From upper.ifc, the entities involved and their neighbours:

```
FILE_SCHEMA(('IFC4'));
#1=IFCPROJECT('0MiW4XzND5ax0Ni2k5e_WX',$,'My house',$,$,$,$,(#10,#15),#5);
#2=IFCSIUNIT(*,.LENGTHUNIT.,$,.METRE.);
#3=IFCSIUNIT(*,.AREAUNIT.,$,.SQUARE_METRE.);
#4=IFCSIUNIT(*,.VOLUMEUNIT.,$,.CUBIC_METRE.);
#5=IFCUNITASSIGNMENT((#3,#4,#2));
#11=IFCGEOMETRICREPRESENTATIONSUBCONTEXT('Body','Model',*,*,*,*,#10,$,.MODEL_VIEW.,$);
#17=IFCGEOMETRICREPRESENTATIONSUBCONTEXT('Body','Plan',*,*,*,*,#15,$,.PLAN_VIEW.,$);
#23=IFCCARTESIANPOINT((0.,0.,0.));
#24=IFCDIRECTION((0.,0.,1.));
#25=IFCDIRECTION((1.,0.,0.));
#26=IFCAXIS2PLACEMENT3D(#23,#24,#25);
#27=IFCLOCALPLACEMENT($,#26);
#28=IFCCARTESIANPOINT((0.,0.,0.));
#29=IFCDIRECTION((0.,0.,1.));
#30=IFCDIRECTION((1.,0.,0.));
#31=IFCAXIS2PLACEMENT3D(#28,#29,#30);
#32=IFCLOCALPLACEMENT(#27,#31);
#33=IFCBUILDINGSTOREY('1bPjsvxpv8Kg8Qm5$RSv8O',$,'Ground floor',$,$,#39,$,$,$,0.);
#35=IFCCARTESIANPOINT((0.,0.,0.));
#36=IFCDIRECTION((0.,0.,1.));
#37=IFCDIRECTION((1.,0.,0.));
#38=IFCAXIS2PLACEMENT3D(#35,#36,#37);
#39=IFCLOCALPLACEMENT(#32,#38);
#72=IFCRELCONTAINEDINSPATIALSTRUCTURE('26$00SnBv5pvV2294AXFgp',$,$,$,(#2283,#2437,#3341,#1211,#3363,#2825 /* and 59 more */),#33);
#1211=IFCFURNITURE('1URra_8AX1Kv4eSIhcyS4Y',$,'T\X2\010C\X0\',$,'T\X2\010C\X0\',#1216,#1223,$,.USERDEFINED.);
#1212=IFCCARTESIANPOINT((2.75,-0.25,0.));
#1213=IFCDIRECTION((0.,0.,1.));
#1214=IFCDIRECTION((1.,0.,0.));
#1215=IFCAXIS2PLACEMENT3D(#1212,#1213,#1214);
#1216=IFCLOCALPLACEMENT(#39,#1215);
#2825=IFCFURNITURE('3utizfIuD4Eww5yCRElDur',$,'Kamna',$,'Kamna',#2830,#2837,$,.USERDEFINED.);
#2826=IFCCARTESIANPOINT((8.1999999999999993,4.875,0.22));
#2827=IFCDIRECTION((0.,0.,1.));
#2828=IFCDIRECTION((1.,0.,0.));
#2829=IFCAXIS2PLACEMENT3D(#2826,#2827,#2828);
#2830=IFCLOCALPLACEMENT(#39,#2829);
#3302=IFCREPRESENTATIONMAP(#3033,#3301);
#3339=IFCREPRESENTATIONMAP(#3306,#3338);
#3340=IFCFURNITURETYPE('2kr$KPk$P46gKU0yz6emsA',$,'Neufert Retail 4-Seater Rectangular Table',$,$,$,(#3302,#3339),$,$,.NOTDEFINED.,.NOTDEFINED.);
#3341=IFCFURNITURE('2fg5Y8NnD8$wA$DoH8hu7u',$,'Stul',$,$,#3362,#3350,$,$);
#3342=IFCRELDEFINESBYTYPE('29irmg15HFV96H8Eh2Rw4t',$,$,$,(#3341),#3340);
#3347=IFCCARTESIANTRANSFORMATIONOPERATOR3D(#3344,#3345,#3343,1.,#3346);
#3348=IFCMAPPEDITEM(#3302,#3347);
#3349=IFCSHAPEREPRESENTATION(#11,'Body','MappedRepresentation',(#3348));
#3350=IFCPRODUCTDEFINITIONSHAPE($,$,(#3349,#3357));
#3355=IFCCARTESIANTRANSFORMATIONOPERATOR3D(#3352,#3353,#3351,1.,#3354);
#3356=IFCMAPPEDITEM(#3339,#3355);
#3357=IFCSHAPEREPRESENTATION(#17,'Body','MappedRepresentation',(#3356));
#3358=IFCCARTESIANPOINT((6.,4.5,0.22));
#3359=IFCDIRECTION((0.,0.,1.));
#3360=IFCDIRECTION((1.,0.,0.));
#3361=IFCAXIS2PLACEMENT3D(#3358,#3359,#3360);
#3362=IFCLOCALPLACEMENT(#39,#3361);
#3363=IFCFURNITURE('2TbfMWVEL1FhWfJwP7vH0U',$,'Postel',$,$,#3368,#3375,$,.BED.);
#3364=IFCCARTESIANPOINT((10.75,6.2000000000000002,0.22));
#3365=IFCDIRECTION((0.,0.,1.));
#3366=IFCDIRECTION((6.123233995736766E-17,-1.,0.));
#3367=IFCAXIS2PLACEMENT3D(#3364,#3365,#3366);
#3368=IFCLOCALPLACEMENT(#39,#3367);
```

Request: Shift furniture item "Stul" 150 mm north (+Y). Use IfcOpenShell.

```python
import ifcopenshell
import ifcopenshell.api.geometry
import ifcopenshell.util.placement

model = ifcopenshell.open("upper.ifc")

item = model.by_guid("2fg5Y8NnD8$wA$DoH8hu7u")
matrix = ifcopenshell.util.placement.get_local_placement(item.ObjectPlacement)
matrix[1, 3] += 0.15
ifcopenshell.api.geometry.edit_object_placement(model, product=item, matrix=matrix, is_si=False)

print(ifcopenshell.util.placement.get_local_placement(item.ObjectPlacement).round(3) + 0.0)

model.write("upper_rev.ifc")
```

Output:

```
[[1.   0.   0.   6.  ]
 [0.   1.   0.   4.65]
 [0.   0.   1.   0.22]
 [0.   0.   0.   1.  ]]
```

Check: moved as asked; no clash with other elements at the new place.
